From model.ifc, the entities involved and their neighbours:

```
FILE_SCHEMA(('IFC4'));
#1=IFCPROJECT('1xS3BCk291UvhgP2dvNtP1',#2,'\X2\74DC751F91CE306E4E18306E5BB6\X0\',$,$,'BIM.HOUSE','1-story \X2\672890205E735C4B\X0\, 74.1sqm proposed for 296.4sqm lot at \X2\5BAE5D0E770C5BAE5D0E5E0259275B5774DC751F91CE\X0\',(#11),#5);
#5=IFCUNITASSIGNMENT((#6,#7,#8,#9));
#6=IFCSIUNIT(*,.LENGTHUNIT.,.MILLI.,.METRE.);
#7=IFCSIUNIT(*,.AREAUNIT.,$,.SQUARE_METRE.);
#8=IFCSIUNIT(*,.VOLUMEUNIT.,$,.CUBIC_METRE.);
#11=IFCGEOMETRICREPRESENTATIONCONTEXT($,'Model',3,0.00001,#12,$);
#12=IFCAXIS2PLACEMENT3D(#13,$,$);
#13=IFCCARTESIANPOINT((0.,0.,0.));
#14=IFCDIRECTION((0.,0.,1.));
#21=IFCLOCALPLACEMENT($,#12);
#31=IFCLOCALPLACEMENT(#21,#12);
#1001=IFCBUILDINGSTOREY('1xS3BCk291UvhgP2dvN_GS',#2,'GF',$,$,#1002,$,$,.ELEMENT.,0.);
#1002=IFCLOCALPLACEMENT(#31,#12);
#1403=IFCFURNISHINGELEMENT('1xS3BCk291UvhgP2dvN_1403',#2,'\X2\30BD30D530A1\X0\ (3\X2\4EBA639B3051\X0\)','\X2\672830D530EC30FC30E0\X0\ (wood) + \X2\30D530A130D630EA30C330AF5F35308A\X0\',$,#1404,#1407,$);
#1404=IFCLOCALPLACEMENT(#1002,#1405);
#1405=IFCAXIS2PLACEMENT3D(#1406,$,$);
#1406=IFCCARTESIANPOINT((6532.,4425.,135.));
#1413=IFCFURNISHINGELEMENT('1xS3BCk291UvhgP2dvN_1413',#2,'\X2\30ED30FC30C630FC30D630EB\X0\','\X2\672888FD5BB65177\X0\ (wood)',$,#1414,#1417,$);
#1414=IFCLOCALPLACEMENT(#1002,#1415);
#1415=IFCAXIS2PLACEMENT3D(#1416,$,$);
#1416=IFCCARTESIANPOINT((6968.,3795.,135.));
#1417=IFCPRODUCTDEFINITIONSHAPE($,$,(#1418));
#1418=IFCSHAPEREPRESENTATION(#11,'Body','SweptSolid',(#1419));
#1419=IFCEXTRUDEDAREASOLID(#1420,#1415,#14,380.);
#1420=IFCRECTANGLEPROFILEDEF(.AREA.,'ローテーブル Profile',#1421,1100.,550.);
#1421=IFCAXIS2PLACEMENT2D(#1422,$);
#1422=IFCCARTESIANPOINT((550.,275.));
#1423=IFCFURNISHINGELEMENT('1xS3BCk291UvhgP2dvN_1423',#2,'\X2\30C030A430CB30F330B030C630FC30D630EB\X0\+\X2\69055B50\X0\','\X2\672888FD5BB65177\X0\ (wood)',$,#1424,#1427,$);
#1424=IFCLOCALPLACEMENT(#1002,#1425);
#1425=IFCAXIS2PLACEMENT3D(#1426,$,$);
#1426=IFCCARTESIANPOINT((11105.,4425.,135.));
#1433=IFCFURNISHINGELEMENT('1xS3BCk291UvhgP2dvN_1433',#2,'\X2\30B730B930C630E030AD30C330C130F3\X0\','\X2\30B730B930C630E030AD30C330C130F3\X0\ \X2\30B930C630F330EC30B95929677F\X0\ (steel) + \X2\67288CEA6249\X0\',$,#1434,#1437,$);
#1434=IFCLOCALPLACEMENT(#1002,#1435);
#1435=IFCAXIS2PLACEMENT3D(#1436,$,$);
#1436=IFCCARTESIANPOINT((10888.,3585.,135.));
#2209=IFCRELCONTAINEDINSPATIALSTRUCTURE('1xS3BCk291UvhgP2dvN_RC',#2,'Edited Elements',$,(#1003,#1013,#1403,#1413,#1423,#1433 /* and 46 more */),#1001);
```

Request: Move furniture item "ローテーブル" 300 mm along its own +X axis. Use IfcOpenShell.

```python
import ifcopenshell
import ifcopenshell.api.geometry
import ifcopenshell.util.placement

model = ifcopenshell.open("model.ifc")

item = model.by_guid("1xS3BCk291UvhgP2dvN_1413")
matrix = ifcopenshell.util.placement.get_local_placement(item.ObjectPlacement)
matrix[:3, 3] += matrix[:3, 0] * 300.0
ifcopenshell.api.geometry.edit_object_placement(model, product=item, matrix=matrix, is_si=False)

print(ifcopenshell.util.placement.get_local_placement(item.ObjectPlacement).round(3) + 0.0)

model.write("model-out.ifc")
```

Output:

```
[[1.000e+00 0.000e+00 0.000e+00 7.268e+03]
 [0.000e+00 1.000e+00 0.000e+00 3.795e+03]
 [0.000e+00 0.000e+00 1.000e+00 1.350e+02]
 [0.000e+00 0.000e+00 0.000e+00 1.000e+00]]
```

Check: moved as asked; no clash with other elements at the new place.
